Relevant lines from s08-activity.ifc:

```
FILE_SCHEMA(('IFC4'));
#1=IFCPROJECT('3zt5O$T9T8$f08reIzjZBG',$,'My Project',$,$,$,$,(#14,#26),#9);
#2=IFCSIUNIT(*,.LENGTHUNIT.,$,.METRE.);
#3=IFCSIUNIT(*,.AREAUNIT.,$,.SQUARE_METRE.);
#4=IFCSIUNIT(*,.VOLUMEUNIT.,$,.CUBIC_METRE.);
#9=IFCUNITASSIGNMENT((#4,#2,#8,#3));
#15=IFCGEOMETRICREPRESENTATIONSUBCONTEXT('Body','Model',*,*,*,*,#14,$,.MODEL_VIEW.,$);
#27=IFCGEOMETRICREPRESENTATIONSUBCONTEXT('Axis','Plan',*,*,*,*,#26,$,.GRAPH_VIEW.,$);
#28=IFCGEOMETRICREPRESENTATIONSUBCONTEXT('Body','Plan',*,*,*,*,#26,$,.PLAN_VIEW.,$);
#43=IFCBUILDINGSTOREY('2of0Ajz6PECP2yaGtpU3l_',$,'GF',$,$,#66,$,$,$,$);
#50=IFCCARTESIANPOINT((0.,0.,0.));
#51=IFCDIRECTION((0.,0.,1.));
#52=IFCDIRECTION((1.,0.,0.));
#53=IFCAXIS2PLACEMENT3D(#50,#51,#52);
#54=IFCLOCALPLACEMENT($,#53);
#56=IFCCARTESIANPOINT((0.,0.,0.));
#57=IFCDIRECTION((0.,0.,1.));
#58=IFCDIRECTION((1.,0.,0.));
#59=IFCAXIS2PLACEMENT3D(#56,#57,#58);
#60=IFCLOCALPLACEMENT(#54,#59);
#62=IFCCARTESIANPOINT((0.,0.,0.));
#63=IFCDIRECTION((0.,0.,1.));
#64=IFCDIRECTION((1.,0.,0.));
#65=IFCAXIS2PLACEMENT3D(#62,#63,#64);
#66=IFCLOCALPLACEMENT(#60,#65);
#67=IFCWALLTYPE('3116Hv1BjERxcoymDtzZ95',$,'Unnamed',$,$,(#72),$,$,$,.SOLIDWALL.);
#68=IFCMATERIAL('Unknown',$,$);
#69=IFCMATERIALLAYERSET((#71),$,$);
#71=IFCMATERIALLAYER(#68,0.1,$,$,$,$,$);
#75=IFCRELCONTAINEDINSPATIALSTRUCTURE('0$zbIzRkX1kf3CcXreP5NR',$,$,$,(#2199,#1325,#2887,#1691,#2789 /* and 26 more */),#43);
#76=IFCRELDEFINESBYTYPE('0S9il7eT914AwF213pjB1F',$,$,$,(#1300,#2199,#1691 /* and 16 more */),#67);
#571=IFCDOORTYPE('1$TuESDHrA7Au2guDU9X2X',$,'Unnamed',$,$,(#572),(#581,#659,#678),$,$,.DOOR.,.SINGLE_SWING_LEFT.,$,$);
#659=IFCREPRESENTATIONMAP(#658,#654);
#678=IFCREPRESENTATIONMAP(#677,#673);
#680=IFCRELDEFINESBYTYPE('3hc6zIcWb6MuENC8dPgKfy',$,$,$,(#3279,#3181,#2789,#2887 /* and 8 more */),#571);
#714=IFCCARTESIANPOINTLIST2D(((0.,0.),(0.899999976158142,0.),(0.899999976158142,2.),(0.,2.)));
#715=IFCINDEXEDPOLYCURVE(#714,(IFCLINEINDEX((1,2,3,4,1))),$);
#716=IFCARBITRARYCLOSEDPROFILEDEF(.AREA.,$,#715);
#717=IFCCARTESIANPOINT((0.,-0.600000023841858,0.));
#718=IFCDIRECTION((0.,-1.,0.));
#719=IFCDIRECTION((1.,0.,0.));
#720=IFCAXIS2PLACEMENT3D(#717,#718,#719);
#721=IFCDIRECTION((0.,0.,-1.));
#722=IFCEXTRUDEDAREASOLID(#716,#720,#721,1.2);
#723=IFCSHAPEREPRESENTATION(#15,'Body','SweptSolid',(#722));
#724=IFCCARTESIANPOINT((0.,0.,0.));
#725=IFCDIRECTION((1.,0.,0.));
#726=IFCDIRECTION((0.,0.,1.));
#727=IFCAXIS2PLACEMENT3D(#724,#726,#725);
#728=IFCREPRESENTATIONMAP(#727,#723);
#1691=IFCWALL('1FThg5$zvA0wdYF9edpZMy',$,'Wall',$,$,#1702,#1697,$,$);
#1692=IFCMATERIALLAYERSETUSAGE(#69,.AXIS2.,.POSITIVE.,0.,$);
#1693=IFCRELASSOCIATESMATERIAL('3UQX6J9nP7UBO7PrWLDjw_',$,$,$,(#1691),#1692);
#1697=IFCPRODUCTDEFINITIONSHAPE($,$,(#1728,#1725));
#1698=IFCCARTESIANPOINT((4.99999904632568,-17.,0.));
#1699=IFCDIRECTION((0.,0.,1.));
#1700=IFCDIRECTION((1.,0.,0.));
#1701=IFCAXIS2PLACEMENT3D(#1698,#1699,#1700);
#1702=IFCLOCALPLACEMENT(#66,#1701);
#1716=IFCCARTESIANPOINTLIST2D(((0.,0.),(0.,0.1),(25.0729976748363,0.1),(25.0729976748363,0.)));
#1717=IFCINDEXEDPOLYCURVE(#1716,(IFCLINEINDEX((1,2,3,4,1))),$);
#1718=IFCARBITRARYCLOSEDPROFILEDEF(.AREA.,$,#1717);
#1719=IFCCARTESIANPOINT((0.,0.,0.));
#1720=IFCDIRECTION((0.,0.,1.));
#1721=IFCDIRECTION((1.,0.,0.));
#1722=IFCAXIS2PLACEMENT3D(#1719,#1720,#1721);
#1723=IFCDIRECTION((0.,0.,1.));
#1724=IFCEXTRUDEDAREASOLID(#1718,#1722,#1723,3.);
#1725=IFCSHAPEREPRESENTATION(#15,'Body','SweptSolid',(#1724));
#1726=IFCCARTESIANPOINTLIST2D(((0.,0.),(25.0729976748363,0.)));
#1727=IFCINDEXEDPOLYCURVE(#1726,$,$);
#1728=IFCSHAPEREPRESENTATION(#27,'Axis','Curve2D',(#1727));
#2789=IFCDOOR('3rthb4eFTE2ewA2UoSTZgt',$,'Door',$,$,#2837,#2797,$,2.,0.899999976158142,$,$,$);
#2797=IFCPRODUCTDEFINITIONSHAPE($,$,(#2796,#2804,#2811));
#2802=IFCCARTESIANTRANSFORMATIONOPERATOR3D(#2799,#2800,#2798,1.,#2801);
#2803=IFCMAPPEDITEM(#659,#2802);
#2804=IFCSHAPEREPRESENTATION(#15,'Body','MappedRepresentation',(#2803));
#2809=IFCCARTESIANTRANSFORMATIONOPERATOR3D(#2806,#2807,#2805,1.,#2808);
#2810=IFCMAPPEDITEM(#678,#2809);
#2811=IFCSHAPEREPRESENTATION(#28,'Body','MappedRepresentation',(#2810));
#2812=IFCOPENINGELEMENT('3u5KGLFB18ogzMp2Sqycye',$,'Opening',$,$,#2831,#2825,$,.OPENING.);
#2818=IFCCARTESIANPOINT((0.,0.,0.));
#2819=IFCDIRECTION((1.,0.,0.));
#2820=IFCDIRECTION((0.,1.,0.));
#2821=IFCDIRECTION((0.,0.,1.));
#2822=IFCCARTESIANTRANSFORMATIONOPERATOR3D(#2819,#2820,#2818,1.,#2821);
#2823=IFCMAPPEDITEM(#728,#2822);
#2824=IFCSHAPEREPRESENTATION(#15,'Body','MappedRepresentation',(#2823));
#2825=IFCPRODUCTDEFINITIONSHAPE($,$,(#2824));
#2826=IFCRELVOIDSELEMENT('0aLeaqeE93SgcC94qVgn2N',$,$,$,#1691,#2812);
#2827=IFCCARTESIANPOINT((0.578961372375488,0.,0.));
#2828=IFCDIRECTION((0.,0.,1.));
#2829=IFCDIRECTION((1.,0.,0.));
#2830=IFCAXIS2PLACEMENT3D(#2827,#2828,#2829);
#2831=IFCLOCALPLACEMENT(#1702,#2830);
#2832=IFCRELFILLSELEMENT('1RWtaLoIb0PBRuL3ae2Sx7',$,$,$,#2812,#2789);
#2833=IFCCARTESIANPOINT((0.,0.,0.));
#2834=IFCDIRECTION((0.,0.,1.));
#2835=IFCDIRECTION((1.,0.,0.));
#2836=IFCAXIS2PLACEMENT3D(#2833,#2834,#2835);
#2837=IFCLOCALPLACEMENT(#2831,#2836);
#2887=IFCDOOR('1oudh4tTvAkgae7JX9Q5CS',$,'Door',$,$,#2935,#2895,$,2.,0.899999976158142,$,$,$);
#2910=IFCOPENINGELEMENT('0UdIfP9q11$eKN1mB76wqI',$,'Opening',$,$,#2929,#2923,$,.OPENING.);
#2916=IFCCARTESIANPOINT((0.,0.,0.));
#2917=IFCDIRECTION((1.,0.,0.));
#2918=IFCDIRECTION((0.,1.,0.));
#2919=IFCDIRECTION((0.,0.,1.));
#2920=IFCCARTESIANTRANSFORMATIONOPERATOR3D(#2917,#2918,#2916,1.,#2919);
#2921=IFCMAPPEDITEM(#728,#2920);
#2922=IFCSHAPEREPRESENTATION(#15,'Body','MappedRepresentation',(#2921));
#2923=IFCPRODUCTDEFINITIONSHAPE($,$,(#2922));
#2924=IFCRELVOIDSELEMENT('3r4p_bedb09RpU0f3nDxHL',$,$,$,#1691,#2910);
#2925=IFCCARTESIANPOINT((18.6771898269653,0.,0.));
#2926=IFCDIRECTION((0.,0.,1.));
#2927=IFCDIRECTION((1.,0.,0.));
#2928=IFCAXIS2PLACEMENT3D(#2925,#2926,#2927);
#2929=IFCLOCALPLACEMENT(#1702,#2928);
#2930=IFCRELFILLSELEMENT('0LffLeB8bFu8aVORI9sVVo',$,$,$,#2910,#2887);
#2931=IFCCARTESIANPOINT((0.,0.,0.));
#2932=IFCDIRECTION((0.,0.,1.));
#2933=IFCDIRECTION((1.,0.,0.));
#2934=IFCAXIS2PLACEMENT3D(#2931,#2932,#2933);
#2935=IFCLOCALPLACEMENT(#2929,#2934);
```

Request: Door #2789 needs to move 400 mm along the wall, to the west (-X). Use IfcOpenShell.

```python
import ifcopenshell
import ifcopenshell.api.geometry
import ifcopenshell.util.placement
import ifcopenshell.util.unit

model = ifcopenshell.open("s08-activity.ifc")
unit_scale = ifcopenshell.util.unit.calculate_unit_scale(model)

door = model.by_guid("3rthb4eFTE2ewA2UoSTZgt")
opening = door.FillsVoids[0].RelatingOpeningElement
wall = opening.VoidsElements[0].RelatingBuildingElement

wall_matrix = ifcopenshell.util.placement.get_local_placement(wall.ObjectPlacement)
shift = wall_matrix[:3, 0] * -0.4 / unit_scale
before = ifcopenshell.util.placement.get_local_placement(door.ObjectPlacement)[:3, 3].copy()

# The door is placed relative to its opening, so it follows when the opening moves.
matrix = ifcopenshell.util.placement.get_local_placement(opening.ObjectPlacement)
matrix[:3, 3] += shift
ifcopenshell.api.geometry.edit_object_placement(
    model, product=opening, matrix=matrix, is_si=False, should_transform_children=True
)

after = ifcopenshell.util.placement.get_local_placement(door.ObjectPlacement)[:3, 3]
print("door moved by", (after - before).round(3) + 0.0)

model.write("s08-activity_edited.ifc")
```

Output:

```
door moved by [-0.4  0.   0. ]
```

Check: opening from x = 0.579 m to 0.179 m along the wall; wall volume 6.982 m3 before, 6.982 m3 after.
